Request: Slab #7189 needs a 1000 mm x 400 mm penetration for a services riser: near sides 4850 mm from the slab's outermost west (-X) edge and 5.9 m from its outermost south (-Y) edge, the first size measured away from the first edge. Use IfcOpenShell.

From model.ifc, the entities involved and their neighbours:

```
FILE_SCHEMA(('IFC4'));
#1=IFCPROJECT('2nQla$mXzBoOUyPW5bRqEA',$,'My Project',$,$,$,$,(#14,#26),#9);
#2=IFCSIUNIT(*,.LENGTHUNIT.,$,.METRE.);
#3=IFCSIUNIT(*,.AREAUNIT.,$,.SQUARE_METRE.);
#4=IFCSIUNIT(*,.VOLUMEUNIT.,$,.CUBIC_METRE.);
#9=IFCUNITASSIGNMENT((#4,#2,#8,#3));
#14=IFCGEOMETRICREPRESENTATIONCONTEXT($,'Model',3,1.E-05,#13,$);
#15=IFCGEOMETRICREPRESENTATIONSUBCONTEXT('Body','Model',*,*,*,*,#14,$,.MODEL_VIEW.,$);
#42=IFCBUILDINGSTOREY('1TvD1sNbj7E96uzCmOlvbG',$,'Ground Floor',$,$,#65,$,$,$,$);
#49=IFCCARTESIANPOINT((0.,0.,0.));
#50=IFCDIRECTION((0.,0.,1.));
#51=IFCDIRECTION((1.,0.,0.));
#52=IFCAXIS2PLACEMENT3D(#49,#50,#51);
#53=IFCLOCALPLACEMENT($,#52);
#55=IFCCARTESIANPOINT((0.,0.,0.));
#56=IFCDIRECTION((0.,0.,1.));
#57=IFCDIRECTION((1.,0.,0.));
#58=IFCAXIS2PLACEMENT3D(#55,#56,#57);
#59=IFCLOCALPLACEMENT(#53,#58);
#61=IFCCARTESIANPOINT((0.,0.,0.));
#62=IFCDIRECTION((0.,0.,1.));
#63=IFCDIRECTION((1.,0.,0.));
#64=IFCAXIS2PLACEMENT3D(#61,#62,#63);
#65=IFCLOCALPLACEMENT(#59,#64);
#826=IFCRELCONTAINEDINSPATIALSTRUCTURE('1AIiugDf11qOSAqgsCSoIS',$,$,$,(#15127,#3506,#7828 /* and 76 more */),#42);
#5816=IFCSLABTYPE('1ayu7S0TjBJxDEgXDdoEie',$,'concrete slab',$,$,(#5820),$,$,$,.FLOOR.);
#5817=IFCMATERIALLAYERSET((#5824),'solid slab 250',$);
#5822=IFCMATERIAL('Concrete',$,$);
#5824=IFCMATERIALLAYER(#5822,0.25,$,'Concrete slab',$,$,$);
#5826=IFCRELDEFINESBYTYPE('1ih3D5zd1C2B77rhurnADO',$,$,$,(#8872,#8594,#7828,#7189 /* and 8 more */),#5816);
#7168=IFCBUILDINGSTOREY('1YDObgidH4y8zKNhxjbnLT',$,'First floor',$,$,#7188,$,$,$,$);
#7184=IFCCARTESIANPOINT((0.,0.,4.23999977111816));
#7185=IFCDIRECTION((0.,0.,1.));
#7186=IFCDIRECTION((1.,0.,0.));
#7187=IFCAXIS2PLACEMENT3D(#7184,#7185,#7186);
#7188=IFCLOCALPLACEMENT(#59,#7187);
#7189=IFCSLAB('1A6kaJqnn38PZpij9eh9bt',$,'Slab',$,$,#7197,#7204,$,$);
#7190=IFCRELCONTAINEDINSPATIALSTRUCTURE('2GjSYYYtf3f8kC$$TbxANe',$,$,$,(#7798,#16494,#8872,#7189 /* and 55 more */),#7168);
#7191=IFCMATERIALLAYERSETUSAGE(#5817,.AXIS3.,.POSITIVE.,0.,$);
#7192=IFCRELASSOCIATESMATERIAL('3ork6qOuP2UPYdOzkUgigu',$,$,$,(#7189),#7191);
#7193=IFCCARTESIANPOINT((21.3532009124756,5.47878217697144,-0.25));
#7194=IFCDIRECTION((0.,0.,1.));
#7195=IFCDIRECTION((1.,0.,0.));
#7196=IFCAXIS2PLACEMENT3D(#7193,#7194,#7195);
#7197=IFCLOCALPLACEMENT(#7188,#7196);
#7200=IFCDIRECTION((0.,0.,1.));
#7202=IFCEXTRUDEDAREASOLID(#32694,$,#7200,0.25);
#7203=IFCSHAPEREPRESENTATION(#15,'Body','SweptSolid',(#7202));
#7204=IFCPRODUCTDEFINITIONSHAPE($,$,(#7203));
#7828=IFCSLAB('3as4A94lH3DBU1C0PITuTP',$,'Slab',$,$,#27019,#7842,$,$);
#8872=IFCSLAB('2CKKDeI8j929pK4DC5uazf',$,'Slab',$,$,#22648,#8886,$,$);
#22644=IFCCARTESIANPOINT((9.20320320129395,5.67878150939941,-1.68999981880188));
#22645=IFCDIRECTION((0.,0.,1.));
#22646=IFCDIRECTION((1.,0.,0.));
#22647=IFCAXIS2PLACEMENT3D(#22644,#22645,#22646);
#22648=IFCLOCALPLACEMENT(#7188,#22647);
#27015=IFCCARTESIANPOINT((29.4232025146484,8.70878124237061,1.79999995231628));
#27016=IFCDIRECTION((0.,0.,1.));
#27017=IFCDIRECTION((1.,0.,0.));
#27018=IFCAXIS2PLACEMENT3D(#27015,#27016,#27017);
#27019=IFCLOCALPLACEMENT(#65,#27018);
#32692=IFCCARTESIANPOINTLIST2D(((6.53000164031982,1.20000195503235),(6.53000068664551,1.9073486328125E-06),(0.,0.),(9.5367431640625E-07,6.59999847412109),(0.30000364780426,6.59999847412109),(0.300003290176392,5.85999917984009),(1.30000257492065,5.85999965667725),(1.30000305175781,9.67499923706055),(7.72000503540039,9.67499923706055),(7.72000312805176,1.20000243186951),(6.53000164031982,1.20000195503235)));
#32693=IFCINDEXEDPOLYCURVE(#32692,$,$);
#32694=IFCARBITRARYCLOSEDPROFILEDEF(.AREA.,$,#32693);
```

```python
import numpy as np
import ifcopenshell
import ifcopenshell.api.feature
import ifcopenshell.api.geometry
import ifcopenshell.api.root
import ifcopenshell.geom
import ifcopenshell.util.placement
import ifcopenshell.util.representation
import ifcopenshell.util.shape
import ifcopenshell.util.unit

model = ifcopenshell.open("model.ifc")
unit_scale = ifcopenshell.util.unit.calculate_unit_scale(model)
settings = ifcopenshell.geom.settings()


def volume(element):
    """Net volume in cubic metres, openings subtracted."""
    shape = ifcopenshell.geom.create_shape(settings, element)
    return ifcopenshell.util.shape.get_volume(shape.geometry)


slab = model.by_id(7189)
before = volume(slab)

# Extent in the slab's own axes, in metres. The edges named are its -X and -Y sides.
slab_shape = ifcopenshell.geom.create_shape(settings, slab)
vertices = ifcopenshell.util.shape.get_vertices(slab_shape.geometry)
x_min, y_min, bottom = vertices.min(axis=0)
top = vertices[:, 2].max()

opening = ifcopenshell.api.root.create_entity(model, ifc_class="IfcOpeningElement", name="Services riser opening", predefined_type="OPENING")
context = ifcopenshell.util.representation.get_context(model, "Model", "Body", "MODEL_VIEW")
width, depth = 1, 0.4
outline = [(0.0, 0.0), (width, 0.0), (width, depth), (0.0, depth), (0.0, 0.0)]
# Overshoot both faces by 50 mm so the cut is clean.
shape = ifcopenshell.api.geometry.add_slab_representation(
    model, context=context, depth=top - bottom + 0.1, polyline=outline
)
ifcopenshell.api.geometry.assign_representation(model, product=opening, representation=shape)

matrix = ifcopenshell.util.placement.get_local_placement(slab.ObjectPlacement)
matrix[:, 3] = matrix @ np.append(np.array([x_min + 4.85, y_min + 5.9, bottom - 0.05]) / unit_scale, 1.0)
ifcopenshell.api.geometry.edit_object_placement(model, product=opening, matrix=matrix, is_si=False)
ifcopenshell.api.feature.add_feature(model, feature=opening, element=slab)

after = volume(slab)

print(f"slab volume {before:.3f} -> {after:.3f} m3")

model.write("model_updated.ifc")
```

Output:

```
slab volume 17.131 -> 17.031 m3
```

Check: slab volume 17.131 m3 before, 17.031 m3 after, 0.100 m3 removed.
